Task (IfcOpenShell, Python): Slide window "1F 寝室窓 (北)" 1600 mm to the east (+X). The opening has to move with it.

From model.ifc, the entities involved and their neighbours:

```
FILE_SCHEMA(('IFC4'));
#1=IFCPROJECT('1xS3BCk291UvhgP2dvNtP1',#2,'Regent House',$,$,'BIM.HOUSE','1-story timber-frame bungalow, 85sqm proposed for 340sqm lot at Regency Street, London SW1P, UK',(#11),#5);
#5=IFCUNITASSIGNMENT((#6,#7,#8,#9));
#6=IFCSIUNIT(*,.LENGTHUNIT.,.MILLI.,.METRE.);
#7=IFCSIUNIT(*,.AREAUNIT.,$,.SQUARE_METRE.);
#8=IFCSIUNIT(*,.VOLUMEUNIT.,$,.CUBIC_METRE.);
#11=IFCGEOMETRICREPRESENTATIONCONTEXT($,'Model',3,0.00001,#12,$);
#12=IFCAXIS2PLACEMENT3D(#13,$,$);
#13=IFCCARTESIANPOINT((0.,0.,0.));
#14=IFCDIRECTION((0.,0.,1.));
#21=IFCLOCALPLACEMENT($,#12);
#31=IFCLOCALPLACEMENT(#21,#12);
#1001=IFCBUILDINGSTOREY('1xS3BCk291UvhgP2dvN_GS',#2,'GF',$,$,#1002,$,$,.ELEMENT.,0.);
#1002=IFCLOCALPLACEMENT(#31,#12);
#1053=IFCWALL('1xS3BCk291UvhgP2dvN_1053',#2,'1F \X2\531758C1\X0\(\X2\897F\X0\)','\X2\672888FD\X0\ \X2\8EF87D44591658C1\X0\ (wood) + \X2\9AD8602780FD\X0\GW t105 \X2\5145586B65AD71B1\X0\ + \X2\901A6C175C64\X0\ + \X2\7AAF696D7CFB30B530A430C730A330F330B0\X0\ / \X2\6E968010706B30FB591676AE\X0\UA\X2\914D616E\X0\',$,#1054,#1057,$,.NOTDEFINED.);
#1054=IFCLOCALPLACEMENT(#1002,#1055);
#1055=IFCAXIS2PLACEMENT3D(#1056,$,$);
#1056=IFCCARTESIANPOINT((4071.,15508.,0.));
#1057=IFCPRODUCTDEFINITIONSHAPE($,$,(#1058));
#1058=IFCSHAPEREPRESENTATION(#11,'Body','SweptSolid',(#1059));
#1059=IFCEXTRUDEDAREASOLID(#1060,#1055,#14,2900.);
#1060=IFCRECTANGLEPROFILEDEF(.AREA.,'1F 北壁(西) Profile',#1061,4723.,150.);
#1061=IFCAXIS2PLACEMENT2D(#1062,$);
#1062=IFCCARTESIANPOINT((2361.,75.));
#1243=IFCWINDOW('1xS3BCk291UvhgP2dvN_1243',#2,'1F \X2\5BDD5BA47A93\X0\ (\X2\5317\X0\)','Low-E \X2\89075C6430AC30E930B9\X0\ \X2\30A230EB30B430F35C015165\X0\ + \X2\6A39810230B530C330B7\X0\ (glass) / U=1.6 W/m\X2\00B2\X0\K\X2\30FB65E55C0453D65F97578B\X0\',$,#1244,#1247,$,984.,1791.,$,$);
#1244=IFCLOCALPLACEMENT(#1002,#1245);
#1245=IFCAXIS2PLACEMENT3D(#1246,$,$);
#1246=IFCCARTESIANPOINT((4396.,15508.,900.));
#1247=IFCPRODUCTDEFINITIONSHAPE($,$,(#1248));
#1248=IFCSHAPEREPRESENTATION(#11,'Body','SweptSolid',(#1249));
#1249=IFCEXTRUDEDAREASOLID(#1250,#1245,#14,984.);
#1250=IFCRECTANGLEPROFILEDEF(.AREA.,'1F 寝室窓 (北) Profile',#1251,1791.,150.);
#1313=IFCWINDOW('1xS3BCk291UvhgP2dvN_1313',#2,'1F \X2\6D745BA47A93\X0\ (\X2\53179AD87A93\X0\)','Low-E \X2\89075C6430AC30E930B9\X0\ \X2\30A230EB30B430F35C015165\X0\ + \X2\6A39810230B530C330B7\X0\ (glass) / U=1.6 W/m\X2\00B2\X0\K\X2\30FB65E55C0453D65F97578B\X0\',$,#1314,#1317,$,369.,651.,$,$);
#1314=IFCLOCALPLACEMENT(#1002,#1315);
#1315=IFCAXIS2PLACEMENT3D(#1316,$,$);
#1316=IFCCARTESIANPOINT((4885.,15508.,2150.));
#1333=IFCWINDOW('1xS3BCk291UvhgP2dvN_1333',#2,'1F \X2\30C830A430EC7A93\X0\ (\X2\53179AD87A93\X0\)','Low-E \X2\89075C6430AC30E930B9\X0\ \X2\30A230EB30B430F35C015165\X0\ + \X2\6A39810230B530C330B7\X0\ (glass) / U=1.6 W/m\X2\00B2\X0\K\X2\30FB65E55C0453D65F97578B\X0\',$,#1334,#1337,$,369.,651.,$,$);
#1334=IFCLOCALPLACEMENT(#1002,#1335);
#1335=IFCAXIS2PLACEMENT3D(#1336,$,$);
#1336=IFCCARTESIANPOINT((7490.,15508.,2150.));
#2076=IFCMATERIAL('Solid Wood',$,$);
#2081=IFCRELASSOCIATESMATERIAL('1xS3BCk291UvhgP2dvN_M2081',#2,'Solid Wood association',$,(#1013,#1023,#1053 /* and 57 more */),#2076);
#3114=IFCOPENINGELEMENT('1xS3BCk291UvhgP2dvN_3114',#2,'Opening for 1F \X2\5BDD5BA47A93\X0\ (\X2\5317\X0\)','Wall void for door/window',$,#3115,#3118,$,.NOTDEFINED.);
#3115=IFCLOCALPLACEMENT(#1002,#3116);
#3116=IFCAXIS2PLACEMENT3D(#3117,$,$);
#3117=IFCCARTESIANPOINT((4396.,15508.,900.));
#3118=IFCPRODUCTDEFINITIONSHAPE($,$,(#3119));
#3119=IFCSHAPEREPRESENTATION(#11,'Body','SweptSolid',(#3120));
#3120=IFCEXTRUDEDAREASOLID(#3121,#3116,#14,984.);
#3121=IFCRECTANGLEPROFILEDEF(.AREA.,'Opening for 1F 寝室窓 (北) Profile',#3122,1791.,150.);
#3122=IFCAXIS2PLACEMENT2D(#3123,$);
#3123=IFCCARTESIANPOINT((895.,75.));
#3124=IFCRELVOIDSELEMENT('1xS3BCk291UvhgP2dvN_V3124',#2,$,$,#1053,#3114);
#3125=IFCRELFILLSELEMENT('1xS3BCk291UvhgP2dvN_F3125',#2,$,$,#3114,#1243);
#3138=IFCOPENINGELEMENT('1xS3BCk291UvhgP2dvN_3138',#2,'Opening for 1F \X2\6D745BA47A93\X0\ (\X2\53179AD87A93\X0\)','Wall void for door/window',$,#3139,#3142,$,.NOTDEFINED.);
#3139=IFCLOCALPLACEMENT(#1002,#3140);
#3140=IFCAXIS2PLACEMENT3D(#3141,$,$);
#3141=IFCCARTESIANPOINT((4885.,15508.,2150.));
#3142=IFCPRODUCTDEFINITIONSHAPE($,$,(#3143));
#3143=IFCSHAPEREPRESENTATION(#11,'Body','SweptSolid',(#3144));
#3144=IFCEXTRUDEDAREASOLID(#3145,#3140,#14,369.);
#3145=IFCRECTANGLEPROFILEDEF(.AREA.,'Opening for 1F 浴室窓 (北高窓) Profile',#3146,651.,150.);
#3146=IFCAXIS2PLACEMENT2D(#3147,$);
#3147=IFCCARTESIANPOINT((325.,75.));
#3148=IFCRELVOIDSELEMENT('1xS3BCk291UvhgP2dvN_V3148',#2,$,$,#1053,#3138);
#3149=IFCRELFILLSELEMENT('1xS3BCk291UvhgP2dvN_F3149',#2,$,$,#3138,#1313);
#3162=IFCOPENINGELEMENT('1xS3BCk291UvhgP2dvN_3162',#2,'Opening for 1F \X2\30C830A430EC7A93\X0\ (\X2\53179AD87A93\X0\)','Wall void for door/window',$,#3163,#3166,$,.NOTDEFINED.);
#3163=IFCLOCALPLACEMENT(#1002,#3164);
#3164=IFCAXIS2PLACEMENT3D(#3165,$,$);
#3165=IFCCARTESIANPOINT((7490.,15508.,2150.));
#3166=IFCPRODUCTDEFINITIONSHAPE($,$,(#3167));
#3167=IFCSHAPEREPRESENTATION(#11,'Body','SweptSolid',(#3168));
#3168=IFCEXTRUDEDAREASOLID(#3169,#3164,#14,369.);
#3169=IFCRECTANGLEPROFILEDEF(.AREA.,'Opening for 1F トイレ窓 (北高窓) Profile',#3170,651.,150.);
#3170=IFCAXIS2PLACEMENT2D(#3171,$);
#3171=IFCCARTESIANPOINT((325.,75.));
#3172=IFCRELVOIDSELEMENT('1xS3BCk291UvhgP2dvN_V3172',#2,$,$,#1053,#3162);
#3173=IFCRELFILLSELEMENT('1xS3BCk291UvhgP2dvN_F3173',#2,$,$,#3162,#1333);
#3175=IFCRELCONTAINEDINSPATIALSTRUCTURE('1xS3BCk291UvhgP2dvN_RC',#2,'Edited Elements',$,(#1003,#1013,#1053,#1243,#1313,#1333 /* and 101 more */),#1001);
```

```python
import ifcopenshell
import ifcopenshell.api.geometry
import ifcopenshell.util.placement

model = ifcopenshell.open("model.ifc")

window = model.by_id(1243)
opening = window.FillsVoids[0].RelatingOpeningElement
wall = opening.VoidsElements[0].RelatingBuildingElement

wall_matrix = ifcopenshell.util.placement.get_local_placement(wall.ObjectPlacement)
shift = wall_matrix[:3, 0] * 1600.0
before = ifcopenshell.util.placement.get_local_placement(window.ObjectPlacement)[:3, 3].copy()

# The window is not placed relative to its opening, so move both.
for product in (opening, window):
    matrix = ifcopenshell.util.placement.get_local_placement(product.ObjectPlacement)
    matrix[:3, 3] += shift
    ifcopenshell.api.geometry.edit_object_placement(model, product=product, matrix=matrix, is_si=False)

after = ifcopenshell.util.placement.get_local_placement(window.ObjectPlacement)[:3, 3]
print("window moved by", (after - before).round(3) + 0.0)

model.write("model-out.ifc")
```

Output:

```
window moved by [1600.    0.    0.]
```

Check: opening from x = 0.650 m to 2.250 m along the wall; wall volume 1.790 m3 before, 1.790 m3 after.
